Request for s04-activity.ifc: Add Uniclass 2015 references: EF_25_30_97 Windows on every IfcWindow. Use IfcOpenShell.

First a look at what the model holds.

```python
import ifcopenshell

model = ifcopenshell.open("s04-activity.ifc")
print(model.schema)
print("classifications:", [c.Name for c in model.by_type("IfcClassification")])
for ifc_class in ("IfcDoor", "IfcRoof", "IfcStair", "IfcWall", "IfcWindow"):
    print(ifc_class, len(model.by_type(ifc_class)))
```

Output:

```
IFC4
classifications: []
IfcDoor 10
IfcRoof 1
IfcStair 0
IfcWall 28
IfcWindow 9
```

```python
import ifcopenshell
import ifcopenshell.api.classification

model = ifcopenshell.open("s04-activity.ifc")

system = ifcopenshell.api.classification.add_classification(model, classification="Uniclass 2015")

codes = {
    "IfcWindow": ("EF_25_30_97", "Windows"),
}
for ifc_class, (code, name) in codes.items():
    products = model.by_type(ifc_class)
    ifcopenshell.api.classification.add_reference(
        model, products=products, classification=system, identification=code, name=name
    )
    print(code, len(products))

model.write("s04-activity_edited.ifc")
```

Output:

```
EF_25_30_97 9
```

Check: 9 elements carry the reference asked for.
